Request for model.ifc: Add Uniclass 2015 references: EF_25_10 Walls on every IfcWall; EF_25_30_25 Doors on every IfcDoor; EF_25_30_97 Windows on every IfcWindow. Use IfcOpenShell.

First a look at what the model holds.

```python
import ifcopenshell

model = ifcopenshell.open("model.ifc")
print(model.schema)
print("classifications:", [c.Name for c in model.by_type("IfcClassification")])
for ifc_class in ("IfcDoor", "IfcRoof", "IfcStair", "IfcWall", "IfcWindow"):
    print(ifc_class, len(model.by_type(ifc_class)))
```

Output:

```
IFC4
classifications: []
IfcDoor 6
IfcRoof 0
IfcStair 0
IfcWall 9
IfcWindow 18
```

```python
import ifcopenshell
import ifcopenshell.api.classification

model = ifcopenshell.open("model.ifc")

system = ifcopenshell.api.classification.add_classification(model, classification="Uniclass 2015")

codes = {
    "IfcWall": ("EF_25_10", "Walls"),
    "IfcDoor": ("EF_25_30_25", "Doors"),
    "IfcWindow": ("EF_25_30_97", "Windows"),
}
for ifc_class, (code, name) in codes.items():
    products = model.by_type(ifc_class)
    ifcopenshell.api.classification.add_reference(
        model, products=products, classification=system, identification=code, name=name
    )
    print(code, len(products))

model.write("model_v2.ifc")
```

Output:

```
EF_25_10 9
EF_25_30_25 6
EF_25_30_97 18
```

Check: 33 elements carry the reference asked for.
